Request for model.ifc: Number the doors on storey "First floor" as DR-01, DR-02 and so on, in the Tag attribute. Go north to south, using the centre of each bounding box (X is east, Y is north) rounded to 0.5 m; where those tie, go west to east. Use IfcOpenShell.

First a look at what the model holds.

```python
import ifcopenshell
import ifcopenshell.util.element
import ifcopenshell.util.placement

model = ifcopenshell.open("model.ifc")
print(model.schema)
storey = next(s for s in model.by_type("IfcBuildingStorey") if s.Name == "First floor")
doors = [e for e in ifcopenshell.util.element.get_decomposition(storey) if e.is_a("IfcDoor")]
for e in sorted(doors, key=lambda e: e.id()):
    origin = ifcopenshell.util.placement.get_local_placement(e.ObjectPlacement)[:3, 3]
    print(e.id(), e.Tag, e.Name, origin.round(2) + 0.0, sep=" | ")
```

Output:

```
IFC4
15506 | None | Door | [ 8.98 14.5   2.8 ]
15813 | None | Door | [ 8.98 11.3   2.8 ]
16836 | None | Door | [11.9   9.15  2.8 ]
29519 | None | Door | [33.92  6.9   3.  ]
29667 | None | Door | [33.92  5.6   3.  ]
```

```python
import ifcopenshell
import ifcopenshell.geom
import ifcopenshell.util.element
import ifcopenshell.util.shape

model = ifcopenshell.open("model.ifc")
settings = ifcopenshell.geom.settings()
settings.set("use-world-coords", True)


def centre(element):
    shape = ifcopenshell.geom.create_shape(settings, element)
    return ifcopenshell.util.shape.get_bbox_centroid(shape.geometry)


storey = next(s for s in model.by_type("IfcBuildingStorey") if s.Name == "First floor")
doors = [e for e in ifcopenshell.util.element.get_decomposition(storey) if e.is_a("IfcDoor")]

# Insertion points can sit at a corner or the storey origin, so sort by the geometry (in metres).
centres = {e: centre(e) for e in doors}
doors.sort(key=lambda e: (-round(centres[e][1] / 0.5), centres[e][0]))

for i, e in enumerate(doors, start=1):
    number = f"DR-{i:02d}"
    e.Tag = number
    print(e.id(), number)

model.write("model_v2.ifc")
```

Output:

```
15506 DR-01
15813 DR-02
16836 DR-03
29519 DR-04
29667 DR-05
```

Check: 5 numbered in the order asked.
